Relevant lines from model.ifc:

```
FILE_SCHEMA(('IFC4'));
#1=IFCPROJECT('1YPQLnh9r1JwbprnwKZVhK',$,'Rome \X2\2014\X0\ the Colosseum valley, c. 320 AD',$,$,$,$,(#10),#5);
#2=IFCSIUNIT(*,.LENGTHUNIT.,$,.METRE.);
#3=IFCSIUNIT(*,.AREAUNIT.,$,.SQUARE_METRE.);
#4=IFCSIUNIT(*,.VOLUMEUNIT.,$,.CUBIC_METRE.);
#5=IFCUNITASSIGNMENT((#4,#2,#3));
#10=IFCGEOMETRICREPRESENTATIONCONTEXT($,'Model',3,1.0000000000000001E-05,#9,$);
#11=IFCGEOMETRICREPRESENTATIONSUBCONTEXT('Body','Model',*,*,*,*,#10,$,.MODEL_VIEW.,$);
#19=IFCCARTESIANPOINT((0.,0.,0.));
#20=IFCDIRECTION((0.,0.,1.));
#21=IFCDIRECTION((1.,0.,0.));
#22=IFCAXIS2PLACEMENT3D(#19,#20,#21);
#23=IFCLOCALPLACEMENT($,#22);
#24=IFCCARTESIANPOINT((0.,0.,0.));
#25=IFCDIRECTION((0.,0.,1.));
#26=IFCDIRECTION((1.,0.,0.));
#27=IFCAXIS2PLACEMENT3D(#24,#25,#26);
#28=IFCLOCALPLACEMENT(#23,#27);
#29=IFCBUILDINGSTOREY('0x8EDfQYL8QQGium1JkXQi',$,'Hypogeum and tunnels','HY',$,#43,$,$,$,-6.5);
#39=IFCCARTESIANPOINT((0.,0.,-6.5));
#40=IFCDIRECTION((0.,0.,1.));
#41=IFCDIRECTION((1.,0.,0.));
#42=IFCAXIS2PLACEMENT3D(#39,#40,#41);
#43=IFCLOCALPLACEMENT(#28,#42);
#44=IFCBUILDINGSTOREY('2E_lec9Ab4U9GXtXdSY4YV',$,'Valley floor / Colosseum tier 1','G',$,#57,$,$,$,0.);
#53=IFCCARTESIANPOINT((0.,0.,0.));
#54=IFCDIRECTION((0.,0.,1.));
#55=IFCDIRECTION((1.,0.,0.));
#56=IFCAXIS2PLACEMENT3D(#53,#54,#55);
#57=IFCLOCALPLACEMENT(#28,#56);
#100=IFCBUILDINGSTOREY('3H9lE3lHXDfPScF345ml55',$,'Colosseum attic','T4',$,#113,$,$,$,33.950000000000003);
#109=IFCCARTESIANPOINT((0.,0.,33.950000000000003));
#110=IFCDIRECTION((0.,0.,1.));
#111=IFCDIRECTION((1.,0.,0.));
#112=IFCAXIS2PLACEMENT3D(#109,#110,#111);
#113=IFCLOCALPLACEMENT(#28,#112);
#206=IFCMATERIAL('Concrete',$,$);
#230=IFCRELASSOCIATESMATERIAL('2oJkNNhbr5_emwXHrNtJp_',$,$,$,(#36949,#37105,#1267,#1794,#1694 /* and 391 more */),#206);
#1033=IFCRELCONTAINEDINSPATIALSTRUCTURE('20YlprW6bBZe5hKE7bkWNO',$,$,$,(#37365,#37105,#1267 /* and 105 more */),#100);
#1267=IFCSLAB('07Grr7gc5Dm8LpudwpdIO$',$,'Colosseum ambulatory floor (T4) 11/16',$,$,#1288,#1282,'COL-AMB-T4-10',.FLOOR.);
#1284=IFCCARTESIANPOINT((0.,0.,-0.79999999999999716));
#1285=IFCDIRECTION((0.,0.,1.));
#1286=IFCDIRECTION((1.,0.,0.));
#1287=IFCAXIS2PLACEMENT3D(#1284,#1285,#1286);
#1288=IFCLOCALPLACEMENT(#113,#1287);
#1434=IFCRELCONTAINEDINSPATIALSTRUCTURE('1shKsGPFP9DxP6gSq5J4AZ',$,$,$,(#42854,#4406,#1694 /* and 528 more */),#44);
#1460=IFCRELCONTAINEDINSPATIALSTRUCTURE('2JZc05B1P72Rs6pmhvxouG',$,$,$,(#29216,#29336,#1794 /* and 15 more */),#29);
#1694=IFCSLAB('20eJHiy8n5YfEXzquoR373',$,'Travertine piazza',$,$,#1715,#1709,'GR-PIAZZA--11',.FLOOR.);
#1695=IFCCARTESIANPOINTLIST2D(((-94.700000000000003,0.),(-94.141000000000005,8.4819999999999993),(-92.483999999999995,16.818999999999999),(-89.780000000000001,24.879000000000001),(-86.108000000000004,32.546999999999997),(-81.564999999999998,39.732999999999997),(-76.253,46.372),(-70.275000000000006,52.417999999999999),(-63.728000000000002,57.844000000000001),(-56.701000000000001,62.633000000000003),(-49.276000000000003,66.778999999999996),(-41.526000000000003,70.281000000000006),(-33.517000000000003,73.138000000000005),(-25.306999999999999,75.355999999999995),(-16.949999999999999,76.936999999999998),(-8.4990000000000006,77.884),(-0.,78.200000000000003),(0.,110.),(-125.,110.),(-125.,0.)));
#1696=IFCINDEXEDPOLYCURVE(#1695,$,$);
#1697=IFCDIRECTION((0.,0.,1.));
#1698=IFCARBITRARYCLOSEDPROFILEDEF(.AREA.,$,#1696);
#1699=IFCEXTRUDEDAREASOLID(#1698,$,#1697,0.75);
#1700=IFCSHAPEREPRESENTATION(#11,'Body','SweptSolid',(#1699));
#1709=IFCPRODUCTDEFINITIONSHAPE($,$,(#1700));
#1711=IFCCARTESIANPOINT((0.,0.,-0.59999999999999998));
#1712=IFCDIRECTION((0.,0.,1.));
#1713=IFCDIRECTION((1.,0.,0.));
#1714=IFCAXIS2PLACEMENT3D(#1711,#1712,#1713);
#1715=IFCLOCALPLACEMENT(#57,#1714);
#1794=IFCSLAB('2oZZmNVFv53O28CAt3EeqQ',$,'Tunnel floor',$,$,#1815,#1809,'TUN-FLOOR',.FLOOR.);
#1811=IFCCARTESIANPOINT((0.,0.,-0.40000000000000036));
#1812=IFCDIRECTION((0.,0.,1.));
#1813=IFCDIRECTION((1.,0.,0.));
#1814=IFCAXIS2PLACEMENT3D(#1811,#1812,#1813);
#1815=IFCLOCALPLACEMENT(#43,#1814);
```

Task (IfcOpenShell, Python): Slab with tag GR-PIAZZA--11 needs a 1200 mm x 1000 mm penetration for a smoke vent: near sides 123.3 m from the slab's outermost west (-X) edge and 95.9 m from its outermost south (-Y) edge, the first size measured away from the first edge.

```python
import numpy as np
import ifcopenshell
import ifcopenshell.api.feature
import ifcopenshell.api.geometry
import ifcopenshell.api.root
import ifcopenshell.geom
import ifcopenshell.util.placement
import ifcopenshell.util.representation
import ifcopenshell.util.shape
import ifcopenshell.util.unit

model = ifcopenshell.open("model.ifc")
unit_scale = ifcopenshell.util.unit.calculate_unit_scale(model)
settings = ifcopenshell.geom.settings()


def volume(element):
    """Net volume in cubic metres, openings subtracted."""
    shape = ifcopenshell.geom.create_shape(settings, element)
    return ifcopenshell.util.shape.get_volume(shape.geometry)


slab = model.by_id(1694)
before = volume(slab)

# Extent in the slab's own axes, in metres. The edges named are its -X and -Y sides.
slab_shape = ifcopenshell.geom.create_shape(settings, slab)
vertices = ifcopenshell.util.shape.get_vertices(slab_shape.geometry)
x_min, y_min, bottom = vertices.min(axis=0)
top = vertices[:, 2].max()

opening = ifcopenshell.api.root.create_entity(model, ifc_class="IfcOpeningElement", name="Smoke vent opening", predefined_type="OPENING")
context = ifcopenshell.util.representation.get_context(model, "Model", "Body", "MODEL_VIEW")
width, depth = 1.2, 1
outline = [(0.0, 0.0), (width, 0.0), (width, depth), (0.0, depth), (0.0, 0.0)]
# Overshoot both faces by 50 mm so the cut is clean.
shape = ifcopenshell.api.geometry.add_slab_representation(
    model, context=context, depth=top - bottom + 0.1, polyline=outline
)
ifcopenshell.api.geometry.assign_representation(model, product=opening, representation=shape)

matrix = ifcopenshell.util.placement.get_local_placement(slab.ObjectPlacement)
matrix[:, 3] = matrix @ np.append(np.array([x_min + 123.3, y_min + 95.9, bottom - 0.05]) / unit_scale, 1.0)
ifcopenshell.api.geometry.edit_object_placement(model, product=opening, matrix=matrix, is_si=False)
ifcopenshell.api.feature.add_feature(model, feature=opening, element=slab)

after = volume(slab)

print(f"slab volume {before:.3f} -> {after:.3f} m3")

model.write("model_rev.ifc")
```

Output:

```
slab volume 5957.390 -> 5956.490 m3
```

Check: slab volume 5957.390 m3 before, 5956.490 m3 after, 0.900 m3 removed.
